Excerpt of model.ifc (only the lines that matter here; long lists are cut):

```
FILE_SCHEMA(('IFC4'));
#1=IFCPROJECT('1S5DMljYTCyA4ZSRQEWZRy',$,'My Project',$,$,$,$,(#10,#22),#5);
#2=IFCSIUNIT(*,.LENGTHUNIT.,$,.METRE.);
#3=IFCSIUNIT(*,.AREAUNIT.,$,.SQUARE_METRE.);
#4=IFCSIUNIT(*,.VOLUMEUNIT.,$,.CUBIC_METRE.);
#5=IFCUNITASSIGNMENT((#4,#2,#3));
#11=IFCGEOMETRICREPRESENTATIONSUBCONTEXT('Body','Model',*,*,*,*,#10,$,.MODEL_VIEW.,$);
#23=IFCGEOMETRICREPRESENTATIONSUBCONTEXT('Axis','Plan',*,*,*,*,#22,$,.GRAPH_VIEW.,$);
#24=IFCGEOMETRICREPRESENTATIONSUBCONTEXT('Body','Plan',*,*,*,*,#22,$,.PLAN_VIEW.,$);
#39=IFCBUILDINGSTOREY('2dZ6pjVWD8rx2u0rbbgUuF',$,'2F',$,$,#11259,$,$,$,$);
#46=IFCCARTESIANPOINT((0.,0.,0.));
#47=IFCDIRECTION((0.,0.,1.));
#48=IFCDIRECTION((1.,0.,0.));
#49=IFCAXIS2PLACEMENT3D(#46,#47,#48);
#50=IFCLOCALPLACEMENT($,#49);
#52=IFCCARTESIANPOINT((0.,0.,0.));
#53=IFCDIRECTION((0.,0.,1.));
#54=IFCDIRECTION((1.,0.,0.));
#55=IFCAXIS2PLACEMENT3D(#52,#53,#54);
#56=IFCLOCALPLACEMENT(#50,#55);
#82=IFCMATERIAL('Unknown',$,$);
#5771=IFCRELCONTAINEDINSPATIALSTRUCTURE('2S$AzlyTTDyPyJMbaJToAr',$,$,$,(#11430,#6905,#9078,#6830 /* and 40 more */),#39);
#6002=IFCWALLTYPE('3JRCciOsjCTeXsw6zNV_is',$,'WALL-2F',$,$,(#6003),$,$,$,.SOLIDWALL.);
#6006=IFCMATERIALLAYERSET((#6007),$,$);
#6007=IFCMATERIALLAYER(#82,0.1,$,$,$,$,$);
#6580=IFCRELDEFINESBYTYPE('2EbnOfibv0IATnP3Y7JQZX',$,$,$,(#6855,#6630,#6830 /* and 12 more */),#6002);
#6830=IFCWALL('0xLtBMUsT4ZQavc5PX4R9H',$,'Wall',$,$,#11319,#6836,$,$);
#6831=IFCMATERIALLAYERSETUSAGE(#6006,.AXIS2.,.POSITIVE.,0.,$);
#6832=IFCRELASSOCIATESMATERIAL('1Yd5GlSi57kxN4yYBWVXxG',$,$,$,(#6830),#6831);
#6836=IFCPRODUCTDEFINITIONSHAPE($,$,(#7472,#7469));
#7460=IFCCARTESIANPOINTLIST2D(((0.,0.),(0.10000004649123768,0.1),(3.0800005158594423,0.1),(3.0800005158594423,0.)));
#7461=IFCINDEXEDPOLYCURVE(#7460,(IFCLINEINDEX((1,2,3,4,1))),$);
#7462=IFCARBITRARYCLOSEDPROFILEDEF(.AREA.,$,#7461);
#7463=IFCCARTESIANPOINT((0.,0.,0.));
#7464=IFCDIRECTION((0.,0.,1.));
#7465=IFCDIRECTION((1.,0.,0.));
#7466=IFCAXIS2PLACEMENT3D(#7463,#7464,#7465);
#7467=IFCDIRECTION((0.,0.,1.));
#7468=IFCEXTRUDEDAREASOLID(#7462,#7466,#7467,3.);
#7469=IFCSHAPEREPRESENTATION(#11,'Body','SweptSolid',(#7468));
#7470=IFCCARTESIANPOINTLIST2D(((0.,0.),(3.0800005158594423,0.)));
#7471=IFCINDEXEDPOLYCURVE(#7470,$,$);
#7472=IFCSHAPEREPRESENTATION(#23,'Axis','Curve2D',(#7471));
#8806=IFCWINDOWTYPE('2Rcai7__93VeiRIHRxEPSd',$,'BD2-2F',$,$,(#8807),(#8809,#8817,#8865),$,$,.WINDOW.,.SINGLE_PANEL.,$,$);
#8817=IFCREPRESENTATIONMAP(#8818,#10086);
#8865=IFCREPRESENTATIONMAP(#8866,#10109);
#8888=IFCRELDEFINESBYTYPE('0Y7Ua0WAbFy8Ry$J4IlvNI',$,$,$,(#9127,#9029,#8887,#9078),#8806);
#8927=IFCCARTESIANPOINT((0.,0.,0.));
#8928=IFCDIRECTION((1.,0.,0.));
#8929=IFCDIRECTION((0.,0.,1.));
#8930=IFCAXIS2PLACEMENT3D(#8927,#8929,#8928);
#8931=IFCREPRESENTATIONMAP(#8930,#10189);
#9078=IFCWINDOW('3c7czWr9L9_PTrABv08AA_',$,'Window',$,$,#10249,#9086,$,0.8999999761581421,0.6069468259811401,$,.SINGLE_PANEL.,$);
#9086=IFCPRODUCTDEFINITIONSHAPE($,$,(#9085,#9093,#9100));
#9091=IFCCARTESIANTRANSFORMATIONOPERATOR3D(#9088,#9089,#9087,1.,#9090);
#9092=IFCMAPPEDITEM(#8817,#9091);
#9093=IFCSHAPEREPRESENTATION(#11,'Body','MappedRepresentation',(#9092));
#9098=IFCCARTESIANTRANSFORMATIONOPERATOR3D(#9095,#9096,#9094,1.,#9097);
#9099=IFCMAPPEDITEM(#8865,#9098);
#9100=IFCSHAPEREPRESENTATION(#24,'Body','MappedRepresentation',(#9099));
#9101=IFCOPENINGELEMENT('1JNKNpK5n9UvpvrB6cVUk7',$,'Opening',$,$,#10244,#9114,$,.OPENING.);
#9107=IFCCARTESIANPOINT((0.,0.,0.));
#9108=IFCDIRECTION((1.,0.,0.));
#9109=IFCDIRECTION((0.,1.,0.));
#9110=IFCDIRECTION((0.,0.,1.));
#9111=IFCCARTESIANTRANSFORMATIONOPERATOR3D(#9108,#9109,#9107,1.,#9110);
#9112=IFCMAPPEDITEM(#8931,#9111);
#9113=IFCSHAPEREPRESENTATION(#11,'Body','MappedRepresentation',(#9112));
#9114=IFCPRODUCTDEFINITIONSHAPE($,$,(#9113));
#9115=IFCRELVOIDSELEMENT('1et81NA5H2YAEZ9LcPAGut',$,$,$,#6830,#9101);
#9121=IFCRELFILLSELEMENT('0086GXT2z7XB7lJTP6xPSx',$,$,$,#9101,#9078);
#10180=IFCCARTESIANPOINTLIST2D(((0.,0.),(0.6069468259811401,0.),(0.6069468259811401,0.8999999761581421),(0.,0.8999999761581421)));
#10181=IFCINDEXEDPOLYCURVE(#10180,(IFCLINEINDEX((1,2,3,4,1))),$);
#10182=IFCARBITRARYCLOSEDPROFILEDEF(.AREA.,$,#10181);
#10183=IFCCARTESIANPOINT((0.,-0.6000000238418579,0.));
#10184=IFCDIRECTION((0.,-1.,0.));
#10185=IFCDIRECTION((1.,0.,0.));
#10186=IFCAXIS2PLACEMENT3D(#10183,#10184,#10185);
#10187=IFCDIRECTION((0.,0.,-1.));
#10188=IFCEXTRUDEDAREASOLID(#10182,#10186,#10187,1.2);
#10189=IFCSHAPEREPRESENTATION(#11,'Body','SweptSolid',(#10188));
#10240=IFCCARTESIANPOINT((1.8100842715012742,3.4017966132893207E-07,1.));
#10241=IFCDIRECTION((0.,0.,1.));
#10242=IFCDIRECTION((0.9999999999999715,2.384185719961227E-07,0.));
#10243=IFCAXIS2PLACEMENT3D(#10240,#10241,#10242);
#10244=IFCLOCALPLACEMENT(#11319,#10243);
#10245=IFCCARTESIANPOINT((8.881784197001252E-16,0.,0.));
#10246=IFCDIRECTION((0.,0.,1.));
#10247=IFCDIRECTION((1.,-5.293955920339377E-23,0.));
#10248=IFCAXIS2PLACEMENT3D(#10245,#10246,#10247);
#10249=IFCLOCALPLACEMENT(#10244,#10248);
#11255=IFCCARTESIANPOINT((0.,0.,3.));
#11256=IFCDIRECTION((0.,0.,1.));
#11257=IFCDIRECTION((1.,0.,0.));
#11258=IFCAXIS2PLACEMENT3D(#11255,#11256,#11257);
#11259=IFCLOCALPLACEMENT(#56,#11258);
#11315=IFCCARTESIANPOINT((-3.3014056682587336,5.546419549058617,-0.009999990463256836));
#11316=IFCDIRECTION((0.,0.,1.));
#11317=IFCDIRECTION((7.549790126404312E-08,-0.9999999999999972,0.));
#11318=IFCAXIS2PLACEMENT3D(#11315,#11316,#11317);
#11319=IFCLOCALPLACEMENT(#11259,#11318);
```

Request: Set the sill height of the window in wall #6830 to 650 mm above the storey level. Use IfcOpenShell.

```python
import numpy as np
import ifcopenshell
import ifcopenshell.api.geometry
import ifcopenshell.geom
import ifcopenshell.util.element
import ifcopenshell.util.placement
import ifcopenshell.util.shape
import ifcopenshell.util.unit

model = ifcopenshell.open("model.ifc")
unit_scale = ifcopenshell.util.unit.calculate_unit_scale(model)

window = model.by_guid("3c7czWr9L9_PTrABv08AA_")
opening = window.FillsVoids[0].RelatingOpeningElement
storey = ifcopenshell.util.element.get_container(window, ifc_class="IfcBuildingStorey")
level = ifcopenshell.util.placement.get_local_placement(storey.ObjectPlacement)[2, 3]

# The opening's origin need not be at the sill, so measure its lowest point.
shape = ifcopenshell.geom.create_shape(ifcopenshell.geom.settings(), opening)
bottom = ifcopenshell.util.shape.get_shape_bottom_elevation(shape, shape.geometry) / unit_scale
dz = level + 0.65 - bottom

shift = np.array([0.0, 0.0, dz])
# The window is placed relative to its opening, so it follows when the opening moves.
matrix = ifcopenshell.util.placement.get_local_placement(opening.ObjectPlacement)
matrix[:3, 3] += shift
ifcopenshell.api.geometry.edit_object_placement(
    model, product=opening, matrix=matrix, is_si=False, should_transform_children=True
)

print(f"moved by {dz * unit_scale:+.3f} m")

model.write("model_edited.ifc")
```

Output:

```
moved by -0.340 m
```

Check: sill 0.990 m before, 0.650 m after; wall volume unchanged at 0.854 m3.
